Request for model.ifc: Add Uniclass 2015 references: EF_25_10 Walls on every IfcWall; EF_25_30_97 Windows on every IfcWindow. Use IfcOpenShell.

First a look at what the model holds.

```python
import ifcopenshell

model = ifcopenshell.open("model.ifc")
print(model.schema)
print("classifications:", [c.Name for c in model.by_type("IfcClassification")])
for ifc_class in ("IfcDoor", "IfcRoof", "IfcStair", "IfcWall", "IfcWindow"):
    print(ifc_class, len(model.by_type(ifc_class)))
```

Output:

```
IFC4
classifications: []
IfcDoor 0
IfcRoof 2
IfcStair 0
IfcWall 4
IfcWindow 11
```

```python
import ifcopenshell
import ifcopenshell.api.classification

model = ifcopenshell.open("model.ifc")

system = ifcopenshell.api.classification.add_classification(model, classification="Uniclass 2015")

codes = {
    "IfcWall": ("EF_25_10", "Walls"),
    "IfcWindow": ("EF_25_30_97", "Windows"),
}
for ifc_class, (code, name) in codes.items():
    products = model.by_type(ifc_class)
    ifcopenshell.api.classification.add_reference(
        model, products=products, classification=system, identification=code, name=name
    )
    print(code, len(products))

model.write("model_edited.ifc")
```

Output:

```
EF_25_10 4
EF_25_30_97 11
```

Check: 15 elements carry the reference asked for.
